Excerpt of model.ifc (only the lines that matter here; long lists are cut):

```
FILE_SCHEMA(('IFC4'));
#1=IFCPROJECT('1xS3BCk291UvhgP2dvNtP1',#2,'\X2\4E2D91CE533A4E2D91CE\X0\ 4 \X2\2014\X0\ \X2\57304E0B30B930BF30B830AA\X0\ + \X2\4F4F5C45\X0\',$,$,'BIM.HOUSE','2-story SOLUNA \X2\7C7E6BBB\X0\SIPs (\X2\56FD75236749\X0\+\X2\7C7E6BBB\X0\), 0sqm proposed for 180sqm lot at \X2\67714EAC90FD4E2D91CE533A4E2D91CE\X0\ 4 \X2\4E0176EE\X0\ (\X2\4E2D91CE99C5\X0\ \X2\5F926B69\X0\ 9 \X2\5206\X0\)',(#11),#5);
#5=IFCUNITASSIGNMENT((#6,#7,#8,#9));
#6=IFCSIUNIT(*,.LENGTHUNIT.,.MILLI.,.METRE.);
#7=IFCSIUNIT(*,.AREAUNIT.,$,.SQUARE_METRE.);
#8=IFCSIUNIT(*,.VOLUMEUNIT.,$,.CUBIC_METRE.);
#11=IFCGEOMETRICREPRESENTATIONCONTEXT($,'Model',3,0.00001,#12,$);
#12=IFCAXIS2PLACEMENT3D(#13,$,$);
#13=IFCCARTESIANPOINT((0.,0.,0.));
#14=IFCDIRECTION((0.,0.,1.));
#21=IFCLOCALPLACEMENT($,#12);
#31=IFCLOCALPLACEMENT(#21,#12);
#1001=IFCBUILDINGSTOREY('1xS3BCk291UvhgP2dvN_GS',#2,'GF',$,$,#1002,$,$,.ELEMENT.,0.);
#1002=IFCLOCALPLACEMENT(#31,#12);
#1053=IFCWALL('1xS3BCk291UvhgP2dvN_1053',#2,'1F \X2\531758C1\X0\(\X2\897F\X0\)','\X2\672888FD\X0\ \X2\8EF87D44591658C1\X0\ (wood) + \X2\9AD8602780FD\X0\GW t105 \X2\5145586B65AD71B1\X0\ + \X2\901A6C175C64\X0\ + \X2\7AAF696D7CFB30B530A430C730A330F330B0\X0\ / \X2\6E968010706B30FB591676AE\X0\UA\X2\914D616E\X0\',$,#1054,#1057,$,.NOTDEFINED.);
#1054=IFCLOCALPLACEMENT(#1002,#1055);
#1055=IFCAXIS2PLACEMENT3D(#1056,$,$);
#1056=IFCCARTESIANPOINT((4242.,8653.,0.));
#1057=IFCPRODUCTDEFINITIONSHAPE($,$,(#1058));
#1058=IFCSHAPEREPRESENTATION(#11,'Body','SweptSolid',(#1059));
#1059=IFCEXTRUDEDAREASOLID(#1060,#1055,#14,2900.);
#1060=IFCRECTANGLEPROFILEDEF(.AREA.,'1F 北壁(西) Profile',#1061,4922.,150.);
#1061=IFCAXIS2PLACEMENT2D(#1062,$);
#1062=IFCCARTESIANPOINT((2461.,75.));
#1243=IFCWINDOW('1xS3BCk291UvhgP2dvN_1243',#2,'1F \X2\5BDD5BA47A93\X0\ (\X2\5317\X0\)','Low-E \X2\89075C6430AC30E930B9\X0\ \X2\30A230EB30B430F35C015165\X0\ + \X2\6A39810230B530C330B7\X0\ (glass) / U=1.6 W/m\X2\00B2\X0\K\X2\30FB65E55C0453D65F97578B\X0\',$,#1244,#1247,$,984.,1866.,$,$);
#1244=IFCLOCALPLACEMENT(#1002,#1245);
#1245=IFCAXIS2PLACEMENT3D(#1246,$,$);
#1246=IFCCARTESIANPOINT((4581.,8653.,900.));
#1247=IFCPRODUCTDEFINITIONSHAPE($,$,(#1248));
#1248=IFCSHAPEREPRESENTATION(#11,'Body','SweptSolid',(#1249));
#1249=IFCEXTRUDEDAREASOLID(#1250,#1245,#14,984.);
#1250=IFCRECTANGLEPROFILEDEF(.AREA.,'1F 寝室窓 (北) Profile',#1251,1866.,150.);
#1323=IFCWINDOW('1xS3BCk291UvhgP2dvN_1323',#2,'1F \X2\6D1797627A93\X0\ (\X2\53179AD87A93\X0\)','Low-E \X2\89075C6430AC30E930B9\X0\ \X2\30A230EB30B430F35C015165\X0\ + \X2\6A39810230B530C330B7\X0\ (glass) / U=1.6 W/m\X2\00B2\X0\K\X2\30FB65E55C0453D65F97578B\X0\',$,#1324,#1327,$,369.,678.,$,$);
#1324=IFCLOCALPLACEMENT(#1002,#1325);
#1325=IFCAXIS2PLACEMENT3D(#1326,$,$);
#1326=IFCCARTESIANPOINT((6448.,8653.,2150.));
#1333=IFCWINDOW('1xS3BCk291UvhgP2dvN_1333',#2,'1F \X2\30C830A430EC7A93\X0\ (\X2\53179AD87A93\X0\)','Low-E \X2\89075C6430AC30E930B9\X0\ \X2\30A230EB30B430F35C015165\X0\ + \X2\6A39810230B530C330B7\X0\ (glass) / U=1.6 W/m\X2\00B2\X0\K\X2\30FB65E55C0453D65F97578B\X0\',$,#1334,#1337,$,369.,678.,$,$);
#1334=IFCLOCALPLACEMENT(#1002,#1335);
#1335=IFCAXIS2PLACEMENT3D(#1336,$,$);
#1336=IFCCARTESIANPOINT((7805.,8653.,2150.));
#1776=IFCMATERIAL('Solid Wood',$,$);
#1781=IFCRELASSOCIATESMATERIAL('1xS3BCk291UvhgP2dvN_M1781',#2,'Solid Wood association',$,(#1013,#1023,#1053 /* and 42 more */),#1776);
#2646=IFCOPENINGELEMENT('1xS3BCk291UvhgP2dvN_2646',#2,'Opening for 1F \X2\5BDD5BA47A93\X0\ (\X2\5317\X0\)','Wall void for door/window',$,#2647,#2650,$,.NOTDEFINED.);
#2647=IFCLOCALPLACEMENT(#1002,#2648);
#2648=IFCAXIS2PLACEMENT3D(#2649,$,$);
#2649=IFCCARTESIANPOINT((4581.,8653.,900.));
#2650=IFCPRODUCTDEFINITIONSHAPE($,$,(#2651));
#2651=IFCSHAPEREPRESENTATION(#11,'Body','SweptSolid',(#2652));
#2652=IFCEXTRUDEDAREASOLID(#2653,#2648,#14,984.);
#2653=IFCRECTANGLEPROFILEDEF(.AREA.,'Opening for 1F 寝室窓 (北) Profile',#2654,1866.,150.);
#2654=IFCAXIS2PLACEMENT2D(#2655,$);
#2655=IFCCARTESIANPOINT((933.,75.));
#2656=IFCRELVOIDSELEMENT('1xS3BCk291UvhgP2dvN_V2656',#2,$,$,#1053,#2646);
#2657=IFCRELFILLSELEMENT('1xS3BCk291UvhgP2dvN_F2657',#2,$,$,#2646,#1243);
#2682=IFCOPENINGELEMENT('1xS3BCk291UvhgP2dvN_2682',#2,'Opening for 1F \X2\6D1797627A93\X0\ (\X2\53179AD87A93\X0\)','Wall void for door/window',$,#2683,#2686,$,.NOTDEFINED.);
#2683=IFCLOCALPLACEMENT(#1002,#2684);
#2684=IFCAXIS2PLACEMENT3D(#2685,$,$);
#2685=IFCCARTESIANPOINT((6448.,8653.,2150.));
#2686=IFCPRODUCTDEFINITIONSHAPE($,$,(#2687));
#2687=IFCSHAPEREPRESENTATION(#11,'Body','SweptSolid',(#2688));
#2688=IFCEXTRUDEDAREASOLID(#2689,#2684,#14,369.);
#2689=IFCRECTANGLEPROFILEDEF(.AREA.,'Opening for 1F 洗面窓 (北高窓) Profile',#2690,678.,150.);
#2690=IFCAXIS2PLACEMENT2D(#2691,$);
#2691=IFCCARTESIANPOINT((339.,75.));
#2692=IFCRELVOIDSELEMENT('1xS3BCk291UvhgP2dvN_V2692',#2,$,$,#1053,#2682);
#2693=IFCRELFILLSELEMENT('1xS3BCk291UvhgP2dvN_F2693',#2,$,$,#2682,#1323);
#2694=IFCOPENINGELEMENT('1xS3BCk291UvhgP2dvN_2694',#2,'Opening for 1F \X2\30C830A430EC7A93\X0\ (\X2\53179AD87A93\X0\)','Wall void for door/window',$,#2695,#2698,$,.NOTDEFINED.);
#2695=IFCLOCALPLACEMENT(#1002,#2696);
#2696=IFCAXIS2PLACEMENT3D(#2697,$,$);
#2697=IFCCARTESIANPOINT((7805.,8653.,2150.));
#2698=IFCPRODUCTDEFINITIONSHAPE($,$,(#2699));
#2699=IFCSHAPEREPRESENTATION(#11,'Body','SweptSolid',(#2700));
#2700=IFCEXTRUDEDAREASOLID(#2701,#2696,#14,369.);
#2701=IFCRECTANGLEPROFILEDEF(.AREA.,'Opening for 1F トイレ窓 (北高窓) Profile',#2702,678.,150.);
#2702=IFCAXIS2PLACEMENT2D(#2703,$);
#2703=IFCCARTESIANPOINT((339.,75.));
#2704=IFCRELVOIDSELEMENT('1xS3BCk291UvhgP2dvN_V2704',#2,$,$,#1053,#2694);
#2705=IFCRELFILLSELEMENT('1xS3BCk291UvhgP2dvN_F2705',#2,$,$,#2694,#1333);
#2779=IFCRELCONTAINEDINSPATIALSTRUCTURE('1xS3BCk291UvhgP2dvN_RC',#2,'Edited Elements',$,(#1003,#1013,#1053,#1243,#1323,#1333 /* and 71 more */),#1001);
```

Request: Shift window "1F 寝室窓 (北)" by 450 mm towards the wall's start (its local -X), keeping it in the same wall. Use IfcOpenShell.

```python
import ifcopenshell
import ifcopenshell.api.geometry
import ifcopenshell.util.placement
import ifcopenshell.util.unit

model = ifcopenshell.open("model.ifc")
unit_scale = ifcopenshell.util.unit.calculate_unit_scale(model)

window = model.by_guid("1xS3BCk291UvhgP2dvN_1243")
opening = window.FillsVoids[0].RelatingOpeningElement
wall = opening.VoidsElements[0].RelatingBuildingElement

wall_matrix = ifcopenshell.util.placement.get_local_placement(wall.ObjectPlacement)
shift = wall_matrix[:3, 0] * -0.45 / unit_scale
before = ifcopenshell.util.placement.get_local_placement(window.ObjectPlacement)[:3, 3].copy()

# The window is not placed relative to its opening, so move both.
for product in (opening, window):
    matrix = ifcopenshell.util.placement.get_local_placement(product.ObjectPlacement)
    matrix[:3, 3] += shift
    ifcopenshell.api.geometry.edit_object_placement(model, product=product, matrix=matrix, is_si=False)

after = ifcopenshell.util.placement.get_local_placement(window.ObjectPlacement)[:3, 3]
print("window moved by", (after - before).round(3) + 0.0)

model.write("model_updated.ifc")
```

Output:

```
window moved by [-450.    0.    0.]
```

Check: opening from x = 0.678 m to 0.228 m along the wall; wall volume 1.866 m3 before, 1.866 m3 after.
